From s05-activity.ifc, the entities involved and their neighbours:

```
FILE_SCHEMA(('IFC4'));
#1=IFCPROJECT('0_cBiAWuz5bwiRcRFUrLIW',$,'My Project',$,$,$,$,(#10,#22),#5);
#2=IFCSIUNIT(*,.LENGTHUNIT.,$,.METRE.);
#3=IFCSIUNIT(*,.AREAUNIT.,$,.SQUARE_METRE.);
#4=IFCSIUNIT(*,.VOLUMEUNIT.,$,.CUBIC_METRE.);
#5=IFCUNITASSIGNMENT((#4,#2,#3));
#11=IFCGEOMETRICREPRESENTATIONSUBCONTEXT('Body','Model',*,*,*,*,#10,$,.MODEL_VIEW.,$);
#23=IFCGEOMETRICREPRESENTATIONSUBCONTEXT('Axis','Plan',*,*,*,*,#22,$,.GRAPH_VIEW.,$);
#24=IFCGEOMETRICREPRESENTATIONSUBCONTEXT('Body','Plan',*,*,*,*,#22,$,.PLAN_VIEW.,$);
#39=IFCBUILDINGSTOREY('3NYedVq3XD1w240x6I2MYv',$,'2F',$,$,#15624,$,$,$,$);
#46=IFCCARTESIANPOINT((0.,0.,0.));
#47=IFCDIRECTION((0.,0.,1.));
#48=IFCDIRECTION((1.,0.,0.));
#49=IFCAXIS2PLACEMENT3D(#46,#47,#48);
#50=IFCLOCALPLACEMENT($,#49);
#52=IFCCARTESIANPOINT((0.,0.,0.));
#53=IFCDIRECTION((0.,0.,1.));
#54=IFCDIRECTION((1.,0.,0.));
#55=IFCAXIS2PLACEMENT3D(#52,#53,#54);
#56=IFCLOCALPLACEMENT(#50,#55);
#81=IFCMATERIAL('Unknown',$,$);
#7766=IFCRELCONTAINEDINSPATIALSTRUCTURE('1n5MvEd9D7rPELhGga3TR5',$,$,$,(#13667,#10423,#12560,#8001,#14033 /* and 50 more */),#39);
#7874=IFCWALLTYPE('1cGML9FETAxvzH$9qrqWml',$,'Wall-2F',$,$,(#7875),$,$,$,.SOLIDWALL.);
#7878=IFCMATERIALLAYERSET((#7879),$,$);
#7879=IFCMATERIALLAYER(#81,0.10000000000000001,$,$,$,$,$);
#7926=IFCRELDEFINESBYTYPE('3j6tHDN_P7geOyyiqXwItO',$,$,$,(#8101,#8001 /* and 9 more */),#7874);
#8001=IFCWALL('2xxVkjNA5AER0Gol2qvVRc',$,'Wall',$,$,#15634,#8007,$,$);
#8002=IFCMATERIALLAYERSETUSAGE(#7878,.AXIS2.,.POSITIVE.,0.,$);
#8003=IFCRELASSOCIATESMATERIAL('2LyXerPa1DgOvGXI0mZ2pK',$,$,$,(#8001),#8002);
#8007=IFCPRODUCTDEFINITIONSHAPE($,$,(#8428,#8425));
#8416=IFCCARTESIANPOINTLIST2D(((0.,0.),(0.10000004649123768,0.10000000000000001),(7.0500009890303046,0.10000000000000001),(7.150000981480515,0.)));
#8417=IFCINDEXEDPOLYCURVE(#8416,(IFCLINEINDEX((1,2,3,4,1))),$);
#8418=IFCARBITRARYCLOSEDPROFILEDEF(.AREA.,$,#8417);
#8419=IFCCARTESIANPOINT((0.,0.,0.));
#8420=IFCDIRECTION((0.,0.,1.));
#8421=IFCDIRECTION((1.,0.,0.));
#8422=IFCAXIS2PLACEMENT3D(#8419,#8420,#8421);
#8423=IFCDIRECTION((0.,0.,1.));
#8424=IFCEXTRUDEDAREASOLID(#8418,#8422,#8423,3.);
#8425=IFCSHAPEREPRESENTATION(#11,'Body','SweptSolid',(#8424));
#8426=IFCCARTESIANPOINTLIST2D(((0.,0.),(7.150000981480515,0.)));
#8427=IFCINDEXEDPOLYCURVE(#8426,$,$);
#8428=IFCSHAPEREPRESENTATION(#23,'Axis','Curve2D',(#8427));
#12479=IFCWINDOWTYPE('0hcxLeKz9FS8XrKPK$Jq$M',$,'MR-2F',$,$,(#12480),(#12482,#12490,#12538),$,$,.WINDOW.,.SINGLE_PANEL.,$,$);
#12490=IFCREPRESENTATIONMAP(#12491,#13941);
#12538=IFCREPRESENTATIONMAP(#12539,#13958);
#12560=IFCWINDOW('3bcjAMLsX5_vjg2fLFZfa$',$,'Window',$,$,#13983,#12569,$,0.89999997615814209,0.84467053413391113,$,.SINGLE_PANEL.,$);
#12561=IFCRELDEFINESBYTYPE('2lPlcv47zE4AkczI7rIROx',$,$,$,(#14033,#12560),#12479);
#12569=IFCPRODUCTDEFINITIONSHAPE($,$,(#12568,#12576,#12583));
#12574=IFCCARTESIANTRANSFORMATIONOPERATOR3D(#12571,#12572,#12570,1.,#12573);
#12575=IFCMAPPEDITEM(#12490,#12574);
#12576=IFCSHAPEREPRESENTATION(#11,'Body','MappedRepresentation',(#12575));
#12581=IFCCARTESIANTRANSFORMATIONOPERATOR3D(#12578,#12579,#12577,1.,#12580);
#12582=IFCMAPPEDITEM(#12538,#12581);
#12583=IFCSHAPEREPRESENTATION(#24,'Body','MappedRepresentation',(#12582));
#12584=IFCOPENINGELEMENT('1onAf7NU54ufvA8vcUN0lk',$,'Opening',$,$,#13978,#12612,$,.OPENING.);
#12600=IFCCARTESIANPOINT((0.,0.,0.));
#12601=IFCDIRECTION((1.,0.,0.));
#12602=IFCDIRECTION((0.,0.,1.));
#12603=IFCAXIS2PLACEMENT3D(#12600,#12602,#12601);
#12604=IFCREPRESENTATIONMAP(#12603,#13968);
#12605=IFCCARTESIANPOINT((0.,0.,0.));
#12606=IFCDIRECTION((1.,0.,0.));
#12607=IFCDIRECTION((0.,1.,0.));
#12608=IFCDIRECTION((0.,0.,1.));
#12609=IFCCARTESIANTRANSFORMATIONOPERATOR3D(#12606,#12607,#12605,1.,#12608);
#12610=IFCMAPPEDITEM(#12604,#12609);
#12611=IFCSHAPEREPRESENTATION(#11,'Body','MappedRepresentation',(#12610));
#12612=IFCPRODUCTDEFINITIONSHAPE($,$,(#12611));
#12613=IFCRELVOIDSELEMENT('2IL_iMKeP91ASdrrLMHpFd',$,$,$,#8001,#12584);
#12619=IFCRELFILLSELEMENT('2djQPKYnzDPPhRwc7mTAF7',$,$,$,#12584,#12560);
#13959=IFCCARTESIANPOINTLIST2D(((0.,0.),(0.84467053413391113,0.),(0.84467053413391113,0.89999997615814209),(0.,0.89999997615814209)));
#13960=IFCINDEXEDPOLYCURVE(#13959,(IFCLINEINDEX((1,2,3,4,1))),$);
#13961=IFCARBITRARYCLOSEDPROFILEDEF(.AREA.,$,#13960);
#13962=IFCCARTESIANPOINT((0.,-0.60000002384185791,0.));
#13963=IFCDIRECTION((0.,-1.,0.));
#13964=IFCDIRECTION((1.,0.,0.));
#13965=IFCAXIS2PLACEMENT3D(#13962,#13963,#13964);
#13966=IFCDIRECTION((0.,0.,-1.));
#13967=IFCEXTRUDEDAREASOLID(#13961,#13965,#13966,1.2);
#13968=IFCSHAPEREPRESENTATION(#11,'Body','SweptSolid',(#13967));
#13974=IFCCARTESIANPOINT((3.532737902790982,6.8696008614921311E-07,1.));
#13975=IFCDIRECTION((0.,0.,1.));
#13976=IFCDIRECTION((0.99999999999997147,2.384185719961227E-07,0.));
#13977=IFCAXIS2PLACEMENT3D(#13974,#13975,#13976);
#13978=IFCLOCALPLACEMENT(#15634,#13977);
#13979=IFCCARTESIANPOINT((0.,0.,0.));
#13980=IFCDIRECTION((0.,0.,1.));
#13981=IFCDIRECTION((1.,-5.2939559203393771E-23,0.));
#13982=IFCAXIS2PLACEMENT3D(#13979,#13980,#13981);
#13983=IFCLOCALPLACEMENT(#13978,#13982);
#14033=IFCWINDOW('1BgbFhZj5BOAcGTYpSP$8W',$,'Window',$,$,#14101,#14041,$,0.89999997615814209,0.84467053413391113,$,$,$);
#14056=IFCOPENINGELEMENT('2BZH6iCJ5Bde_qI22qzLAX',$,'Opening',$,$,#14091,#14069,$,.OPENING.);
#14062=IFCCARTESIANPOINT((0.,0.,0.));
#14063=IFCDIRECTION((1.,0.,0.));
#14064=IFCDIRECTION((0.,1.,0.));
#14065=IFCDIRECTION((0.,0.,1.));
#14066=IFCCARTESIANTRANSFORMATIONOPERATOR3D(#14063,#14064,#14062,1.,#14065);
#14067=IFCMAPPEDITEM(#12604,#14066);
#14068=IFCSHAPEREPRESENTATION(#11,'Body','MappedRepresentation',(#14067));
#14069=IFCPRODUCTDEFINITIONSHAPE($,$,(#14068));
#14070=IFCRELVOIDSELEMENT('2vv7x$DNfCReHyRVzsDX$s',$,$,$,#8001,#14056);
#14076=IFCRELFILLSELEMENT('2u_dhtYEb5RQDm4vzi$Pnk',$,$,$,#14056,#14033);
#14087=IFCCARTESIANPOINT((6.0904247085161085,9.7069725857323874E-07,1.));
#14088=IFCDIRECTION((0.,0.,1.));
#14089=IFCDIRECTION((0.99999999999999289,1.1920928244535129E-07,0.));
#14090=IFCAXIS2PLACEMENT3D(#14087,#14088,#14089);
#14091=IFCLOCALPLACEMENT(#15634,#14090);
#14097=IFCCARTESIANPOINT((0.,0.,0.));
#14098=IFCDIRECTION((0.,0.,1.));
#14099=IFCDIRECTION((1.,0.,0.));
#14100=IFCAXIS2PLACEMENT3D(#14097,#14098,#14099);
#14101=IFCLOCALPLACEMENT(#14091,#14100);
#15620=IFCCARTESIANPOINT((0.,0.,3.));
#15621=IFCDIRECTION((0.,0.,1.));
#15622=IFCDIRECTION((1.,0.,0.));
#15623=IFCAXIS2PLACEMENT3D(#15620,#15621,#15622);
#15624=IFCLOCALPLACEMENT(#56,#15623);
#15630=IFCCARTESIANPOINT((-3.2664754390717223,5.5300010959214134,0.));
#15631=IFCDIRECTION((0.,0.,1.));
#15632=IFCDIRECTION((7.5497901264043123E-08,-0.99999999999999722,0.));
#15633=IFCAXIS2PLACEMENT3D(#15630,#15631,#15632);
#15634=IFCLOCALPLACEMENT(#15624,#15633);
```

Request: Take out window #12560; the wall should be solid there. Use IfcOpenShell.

```python
import ifcopenshell
import ifcopenshell.api.feature
import ifcopenshell.api.root
import ifcopenshell.geom
import ifcopenshell.util.shape

model = ifcopenshell.open("s05-activity.ifc")
settings = ifcopenshell.geom.settings()


def volume(element):
    """Net volume in cubic metres, openings subtracted."""
    shape = ifcopenshell.geom.create_shape(settings, element)
    return ifcopenshell.util.shape.get_volume(shape.geometry)


window = model.by_guid("3bcjAMLsX5_vjg2fLFZfa$")
opening = window.FillsVoids[0].RelatingOpeningElement
wall = opening.VoidsElements[0].RelatingBuildingElement
before = volume(wall)

ifcopenshell.api.root.remove_product(model, product=window)
ifcopenshell.api.feature.remove_feature(model, feature=opening)

after = volume(wall)

print(f"wall volume {before:.3f} -> {after:.3f} m3")

model.write("s05-activity_v2.ifc")
```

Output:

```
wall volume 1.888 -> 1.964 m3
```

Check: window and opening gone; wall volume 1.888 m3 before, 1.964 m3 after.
